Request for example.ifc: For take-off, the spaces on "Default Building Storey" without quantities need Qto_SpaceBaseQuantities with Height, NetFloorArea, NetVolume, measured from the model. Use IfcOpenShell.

First a look at what the model holds.

```python
import ifcopenshell
import ifcopenshell.util.element
import ifcopenshell.util.unit

model = ifcopenshell.open("example.ifc")
print(model.schema)
for unit_type in ("LENGTHUNIT", "AREAUNIT", "VOLUMEUNIT"):
    print(unit_type, ifcopenshell.util.unit.calculate_unit_scale(model, unit_type))
storey = next(s for s in model.by_type("IfcBuildingStorey") if s.Name == "Default Building Storey")
spaces = [e for e in ifcopenshell.util.element.get_decomposition(storey) if e.is_a("IfcSpace")]
for e in sorted(spaces, key=lambda e: e.id()):
    print(e.id(), e.is_a(), e.Name, list(ifcopenshell.util.element.get_psets(e, qtos_only=True)), sep=" | ")
```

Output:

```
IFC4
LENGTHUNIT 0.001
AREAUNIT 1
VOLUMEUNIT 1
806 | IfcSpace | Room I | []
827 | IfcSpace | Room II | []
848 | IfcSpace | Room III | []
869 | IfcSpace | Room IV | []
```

```python
import ifcopenshell
import ifcopenshell.api.pset
import ifcopenshell.geom
import ifcopenshell.util.element
import ifcopenshell.util.shape
import ifcopenshell.util.unit

model = ifcopenshell.open("example.ifc")
unit_scale = ifcopenshell.util.unit.calculate_unit_scale(model)
area_scale = ifcopenshell.util.unit.calculate_unit_scale(model, "AREAUNIT")
volume_scale = ifcopenshell.util.unit.calculate_unit_scale(model, "VOLUMEUNIT")
settings = ifcopenshell.geom.settings()

storey = next(s for s in model.by_type("IfcBuildingStorey") if s.Name == "Default Building Storey")
spaces = [e for e in ifcopenshell.util.element.get_decomposition(storey) if e.is_a("IfcSpace")]

for e in sorted(spaces, key=lambda e: e.id()):
    if ifcopenshell.util.element.get_psets(e, qtos_only=True, should_inherit=False):
        continue
    # Geometry comes back in metres, in the element's own axes.
    shape = ifcopenshell.geom.create_shape(settings, e)
    values = {
        "Height": ifcopenshell.util.shape.get_z(shape.geometry) / unit_scale,
        "NetFloorArea": ifcopenshell.util.shape.get_footprint_area(shape.geometry) / area_scale,
        "NetVolume": ifcopenshell.util.shape.get_volume(shape.geometry) / volume_scale,
    }
    qto = ifcopenshell.api.pset.add_qto(model, product=e, name="Qto_SpaceBaseQuantities")
    ifcopenshell.api.pset.edit_qto(model, qto=qto, properties=values)
    print(e.id(), {k: round(v, 3) for k, v in values.items()})

model.write("example_rev.ifc")
```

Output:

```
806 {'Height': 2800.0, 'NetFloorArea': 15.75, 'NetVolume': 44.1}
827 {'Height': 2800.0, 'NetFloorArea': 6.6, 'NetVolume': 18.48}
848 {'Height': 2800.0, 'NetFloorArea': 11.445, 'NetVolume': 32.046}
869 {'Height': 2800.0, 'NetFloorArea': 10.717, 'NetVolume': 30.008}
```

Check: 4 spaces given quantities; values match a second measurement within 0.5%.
